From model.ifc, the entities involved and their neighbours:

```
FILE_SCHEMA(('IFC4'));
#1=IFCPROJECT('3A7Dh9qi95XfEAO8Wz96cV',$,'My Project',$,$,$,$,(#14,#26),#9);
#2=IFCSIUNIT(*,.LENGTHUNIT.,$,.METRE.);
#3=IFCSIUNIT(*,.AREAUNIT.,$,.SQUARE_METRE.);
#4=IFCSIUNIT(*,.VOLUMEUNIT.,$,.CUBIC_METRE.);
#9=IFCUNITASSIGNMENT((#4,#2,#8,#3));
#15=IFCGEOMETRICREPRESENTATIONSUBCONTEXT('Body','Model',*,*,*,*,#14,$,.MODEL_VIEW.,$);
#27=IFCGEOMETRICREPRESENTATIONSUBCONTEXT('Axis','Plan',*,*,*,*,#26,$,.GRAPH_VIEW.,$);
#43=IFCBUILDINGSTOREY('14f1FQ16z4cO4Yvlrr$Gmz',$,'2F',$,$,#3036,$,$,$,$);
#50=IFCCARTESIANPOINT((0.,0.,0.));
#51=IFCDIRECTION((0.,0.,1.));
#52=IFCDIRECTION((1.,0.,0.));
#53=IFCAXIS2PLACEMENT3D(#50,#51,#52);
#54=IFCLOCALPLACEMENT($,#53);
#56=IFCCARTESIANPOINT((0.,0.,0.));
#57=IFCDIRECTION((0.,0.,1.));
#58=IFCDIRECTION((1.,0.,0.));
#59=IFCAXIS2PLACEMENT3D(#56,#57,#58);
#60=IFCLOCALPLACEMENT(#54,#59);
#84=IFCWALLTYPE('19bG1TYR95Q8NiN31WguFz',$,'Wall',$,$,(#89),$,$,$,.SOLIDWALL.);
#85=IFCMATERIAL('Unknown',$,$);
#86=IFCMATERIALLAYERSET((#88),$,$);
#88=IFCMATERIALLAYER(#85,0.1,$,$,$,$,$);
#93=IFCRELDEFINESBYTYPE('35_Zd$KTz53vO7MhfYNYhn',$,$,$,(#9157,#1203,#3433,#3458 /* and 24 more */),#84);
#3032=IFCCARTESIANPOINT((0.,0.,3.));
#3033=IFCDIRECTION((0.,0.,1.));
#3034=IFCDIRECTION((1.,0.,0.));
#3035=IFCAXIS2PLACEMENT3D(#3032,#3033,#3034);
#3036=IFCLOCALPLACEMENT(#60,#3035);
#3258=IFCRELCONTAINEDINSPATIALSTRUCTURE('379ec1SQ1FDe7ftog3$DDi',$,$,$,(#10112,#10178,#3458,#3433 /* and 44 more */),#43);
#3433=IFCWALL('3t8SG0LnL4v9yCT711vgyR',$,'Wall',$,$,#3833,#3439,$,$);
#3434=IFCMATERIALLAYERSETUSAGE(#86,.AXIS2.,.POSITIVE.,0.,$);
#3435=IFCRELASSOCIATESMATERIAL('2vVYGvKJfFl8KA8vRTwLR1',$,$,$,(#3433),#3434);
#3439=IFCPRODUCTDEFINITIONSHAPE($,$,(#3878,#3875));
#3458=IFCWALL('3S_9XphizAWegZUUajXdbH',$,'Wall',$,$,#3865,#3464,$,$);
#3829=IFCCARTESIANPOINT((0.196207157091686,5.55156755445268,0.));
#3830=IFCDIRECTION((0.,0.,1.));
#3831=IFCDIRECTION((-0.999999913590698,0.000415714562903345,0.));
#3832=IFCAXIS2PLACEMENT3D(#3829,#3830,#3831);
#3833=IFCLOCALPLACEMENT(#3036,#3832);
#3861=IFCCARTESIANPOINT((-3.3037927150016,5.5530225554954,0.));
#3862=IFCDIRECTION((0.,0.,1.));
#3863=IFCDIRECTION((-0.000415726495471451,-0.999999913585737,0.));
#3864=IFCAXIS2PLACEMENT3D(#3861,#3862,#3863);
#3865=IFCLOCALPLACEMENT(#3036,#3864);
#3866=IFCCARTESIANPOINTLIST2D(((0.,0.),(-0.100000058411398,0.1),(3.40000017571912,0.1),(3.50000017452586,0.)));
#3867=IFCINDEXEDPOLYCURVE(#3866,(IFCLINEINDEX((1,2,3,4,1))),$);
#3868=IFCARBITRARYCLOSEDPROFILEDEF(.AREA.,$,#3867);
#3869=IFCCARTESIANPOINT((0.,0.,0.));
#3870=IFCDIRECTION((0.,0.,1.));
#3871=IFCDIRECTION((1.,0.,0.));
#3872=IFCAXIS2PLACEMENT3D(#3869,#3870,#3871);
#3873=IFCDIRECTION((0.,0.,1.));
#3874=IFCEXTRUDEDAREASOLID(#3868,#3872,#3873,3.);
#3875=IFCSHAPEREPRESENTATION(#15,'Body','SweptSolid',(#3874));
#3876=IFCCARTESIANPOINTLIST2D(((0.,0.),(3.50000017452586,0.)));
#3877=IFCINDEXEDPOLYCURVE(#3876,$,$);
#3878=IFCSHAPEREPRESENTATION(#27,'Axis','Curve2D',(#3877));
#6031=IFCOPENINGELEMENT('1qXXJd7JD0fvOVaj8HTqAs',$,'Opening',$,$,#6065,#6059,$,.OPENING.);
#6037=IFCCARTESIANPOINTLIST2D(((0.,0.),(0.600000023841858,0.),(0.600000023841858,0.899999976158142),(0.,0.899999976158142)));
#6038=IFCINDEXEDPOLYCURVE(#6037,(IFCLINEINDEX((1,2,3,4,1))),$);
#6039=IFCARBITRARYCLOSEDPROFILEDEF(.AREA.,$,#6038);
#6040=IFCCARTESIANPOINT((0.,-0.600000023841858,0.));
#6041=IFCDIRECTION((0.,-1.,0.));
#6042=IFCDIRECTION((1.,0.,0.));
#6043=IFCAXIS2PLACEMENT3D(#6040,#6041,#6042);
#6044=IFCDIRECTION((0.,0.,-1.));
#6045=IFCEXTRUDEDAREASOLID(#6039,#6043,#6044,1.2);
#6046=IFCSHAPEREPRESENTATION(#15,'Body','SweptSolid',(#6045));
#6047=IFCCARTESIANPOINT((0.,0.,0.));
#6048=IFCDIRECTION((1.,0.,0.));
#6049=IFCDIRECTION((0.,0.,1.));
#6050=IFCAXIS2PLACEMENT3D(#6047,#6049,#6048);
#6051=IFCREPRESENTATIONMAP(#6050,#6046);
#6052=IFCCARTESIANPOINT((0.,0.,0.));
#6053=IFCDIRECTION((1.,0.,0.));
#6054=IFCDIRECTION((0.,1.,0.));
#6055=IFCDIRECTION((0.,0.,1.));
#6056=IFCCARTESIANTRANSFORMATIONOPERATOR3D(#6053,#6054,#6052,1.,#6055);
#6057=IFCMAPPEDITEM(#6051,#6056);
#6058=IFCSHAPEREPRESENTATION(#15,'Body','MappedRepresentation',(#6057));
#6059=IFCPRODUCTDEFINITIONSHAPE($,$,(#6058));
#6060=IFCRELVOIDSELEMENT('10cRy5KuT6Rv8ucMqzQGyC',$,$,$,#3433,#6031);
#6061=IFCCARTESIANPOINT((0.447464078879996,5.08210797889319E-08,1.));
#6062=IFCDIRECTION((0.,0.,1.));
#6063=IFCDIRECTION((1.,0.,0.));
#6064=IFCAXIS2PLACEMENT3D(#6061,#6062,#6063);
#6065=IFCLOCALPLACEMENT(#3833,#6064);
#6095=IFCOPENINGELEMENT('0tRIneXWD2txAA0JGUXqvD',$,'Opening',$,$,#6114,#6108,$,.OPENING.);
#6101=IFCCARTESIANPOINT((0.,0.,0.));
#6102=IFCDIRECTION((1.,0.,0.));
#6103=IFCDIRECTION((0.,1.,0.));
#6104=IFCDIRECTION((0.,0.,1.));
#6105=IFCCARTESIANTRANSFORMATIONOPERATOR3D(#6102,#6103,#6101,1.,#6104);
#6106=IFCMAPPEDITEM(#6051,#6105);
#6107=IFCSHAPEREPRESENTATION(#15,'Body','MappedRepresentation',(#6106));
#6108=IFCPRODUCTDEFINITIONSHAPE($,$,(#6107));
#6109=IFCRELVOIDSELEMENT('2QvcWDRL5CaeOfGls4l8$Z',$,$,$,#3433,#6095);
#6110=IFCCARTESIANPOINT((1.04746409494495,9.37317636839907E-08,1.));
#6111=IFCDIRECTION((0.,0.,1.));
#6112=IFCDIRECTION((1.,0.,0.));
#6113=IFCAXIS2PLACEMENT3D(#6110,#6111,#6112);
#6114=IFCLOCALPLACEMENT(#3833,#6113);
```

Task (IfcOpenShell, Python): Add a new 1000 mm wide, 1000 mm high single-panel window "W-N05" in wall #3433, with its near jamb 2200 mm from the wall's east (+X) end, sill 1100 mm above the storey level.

```python
import numpy as np
import ifcopenshell
import ifcopenshell.api.feature
import ifcopenshell.api.geometry
import ifcopenshell.api.root
import ifcopenshell.api.spatial
import ifcopenshell.geom
import ifcopenshell.util.element
import ifcopenshell.util.placement
import ifcopenshell.util.representation
import ifcopenshell.util.shape
import ifcopenshell.util.unit

model = ifcopenshell.open("model.ifc")
unit_scale = ifcopenshell.util.unit.calculate_unit_scale(model)
settings = ifcopenshell.geom.settings()


def volume(element):
    """Net volume in cubic metres, openings subtracted."""
    shape = ifcopenshell.geom.create_shape(settings, element)
    return ifcopenshell.util.shape.get_volume(shape.geometry)


wall = model.by_guid("3t8SG0LnL4v9yCT711vgyR")
storey = ifcopenshell.util.element.get_container(wall, ifc_class="IfcBuildingStorey")
context = ifcopenshell.util.representation.get_context(model, "Model", "Body", "MODEL_VIEW")
before = volume(wall)

width, height, from_end, sill = 1, 1, 2.2, 1.1  # metres

# The wall runs along its own X axis, and the end named is its -X end.
wall_shape = ifcopenshell.geom.create_shape(settings, wall)
x, y, z = ifcopenshell.util.shape.get_vertices(wall_shape.geometry).T
start = x.min() + from_end
face, thickness = float(y.min()), float(y.max() - y.min())
wall_matrix = ifcopenshell.util.placement.get_local_placement(wall.ObjectPlacement)
level = ifcopenshell.util.placement.get_local_placement(storey.ObjectPlacement)[2, 3]


def in_wall(x, y):
    """Placement at x, y metres in the wall's axes, at sill height."""
    matrix = wall_matrix.copy()
    matrix[:, 3] = wall_matrix @ np.array([x / unit_scale, y / unit_scale, 0.0, 1.0])
    matrix[2, 3] = level + sill / unit_scale
    return matrix


# Opening: a box that overshoots both wall faces by 50 mm.
opening = ifcopenshell.api.root.create_entity(model, ifc_class="IfcOpeningElement", predefined_type="OPENING")
box = ifcopenshell.api.geometry.add_wall_representation(
    model, context=context, length=width, height=height, thickness=thickness + 0.1
)
ifcopenshell.api.geometry.assign_representation(model, product=opening, representation=box)
ifcopenshell.api.geometry.edit_object_placement(model, product=opening, matrix=in_wall(start, face - 0.05), is_si=False)
ifcopenshell.api.feature.add_feature(model, feature=opening, element=wall)

window = ifcopenshell.api.root.create_entity(model, ifc_class="IfcWindow", name="W-N05", predefined_type="WINDOW")
window.OverallWidth, window.OverallHeight = width / unit_scale, height / unit_scale
window.PartitioningType = "SINGLE_PANEL"
body = ifcopenshell.api.geometry.add_window_representation(
    model,
    context=context,
    overall_width=window.OverallWidth,
    overall_height=window.OverallHeight,
    partition_type="SINGLE_PANEL",
)
ifcopenshell.api.geometry.assign_representation(model, product=window, representation=body)
ifcopenshell.api.spatial.assign_container(model, products=[window], relating_structure=storey)
ifcopenshell.api.feature.add_filling(model, opening=opening, element=window)

# Centre the window in the wall's thickness.
ifcopenshell.api.geometry.edit_object_placement(model, product=window, matrix=in_wall(start, face), is_si=False)
window_shape = ifcopenshell.geom.create_shape(settings, window)
depth = ifcopenshell.util.shape.get_vertices(window_shape.geometry)[:, 1]
offset = face + thickness / 2 - (depth.min() + depth.max()) / 2
ifcopenshell.api.geometry.edit_object_placement(model, product=window, matrix=in_wall(start, offset), is_si=False)

after = volume(wall)

print(f"wall volume {before:.3f} -> {after:.3f} m3")

model.write("model-out.ifc")
```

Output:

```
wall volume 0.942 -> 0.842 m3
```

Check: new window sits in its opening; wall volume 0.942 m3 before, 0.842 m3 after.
